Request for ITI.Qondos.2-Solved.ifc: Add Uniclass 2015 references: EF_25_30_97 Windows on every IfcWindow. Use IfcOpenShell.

First a look at what the model holds.

```python
import ifcopenshell

model = ifcopenshell.open("ITI.Qondos.2-Solved.ifc")
print(model.schema)
print("classifications:", [c.Name for c in model.by_type("IfcClassification")])
for ifc_class in ("IfcDoor", "IfcRoof", "IfcStair", "IfcWall", "IfcWindow"):
    print(ifc_class, len(model.by_type(ifc_class)))
```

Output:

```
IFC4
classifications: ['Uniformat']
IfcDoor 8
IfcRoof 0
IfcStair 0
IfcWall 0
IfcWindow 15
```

```python
import ifcopenshell
import ifcopenshell.api.classification

model = ifcopenshell.open("ITI.Qondos.2-Solved.ifc")

system = ifcopenshell.api.classification.add_classification(model, classification="Uniclass 2015")

codes = {
    "IfcWindow": ("EF_25_30_97", "Windows"),
}
for ifc_class, (code, name) in codes.items():
    products = model.by_type(ifc_class)
    ifcopenshell.api.classification.add_reference(
        model, products=products, classification=system, identification=code, name=name
    )
    print(code, len(products))

model.write("ITI.Qondos.2-Solved_updated.ifc")
```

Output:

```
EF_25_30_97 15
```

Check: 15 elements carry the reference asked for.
